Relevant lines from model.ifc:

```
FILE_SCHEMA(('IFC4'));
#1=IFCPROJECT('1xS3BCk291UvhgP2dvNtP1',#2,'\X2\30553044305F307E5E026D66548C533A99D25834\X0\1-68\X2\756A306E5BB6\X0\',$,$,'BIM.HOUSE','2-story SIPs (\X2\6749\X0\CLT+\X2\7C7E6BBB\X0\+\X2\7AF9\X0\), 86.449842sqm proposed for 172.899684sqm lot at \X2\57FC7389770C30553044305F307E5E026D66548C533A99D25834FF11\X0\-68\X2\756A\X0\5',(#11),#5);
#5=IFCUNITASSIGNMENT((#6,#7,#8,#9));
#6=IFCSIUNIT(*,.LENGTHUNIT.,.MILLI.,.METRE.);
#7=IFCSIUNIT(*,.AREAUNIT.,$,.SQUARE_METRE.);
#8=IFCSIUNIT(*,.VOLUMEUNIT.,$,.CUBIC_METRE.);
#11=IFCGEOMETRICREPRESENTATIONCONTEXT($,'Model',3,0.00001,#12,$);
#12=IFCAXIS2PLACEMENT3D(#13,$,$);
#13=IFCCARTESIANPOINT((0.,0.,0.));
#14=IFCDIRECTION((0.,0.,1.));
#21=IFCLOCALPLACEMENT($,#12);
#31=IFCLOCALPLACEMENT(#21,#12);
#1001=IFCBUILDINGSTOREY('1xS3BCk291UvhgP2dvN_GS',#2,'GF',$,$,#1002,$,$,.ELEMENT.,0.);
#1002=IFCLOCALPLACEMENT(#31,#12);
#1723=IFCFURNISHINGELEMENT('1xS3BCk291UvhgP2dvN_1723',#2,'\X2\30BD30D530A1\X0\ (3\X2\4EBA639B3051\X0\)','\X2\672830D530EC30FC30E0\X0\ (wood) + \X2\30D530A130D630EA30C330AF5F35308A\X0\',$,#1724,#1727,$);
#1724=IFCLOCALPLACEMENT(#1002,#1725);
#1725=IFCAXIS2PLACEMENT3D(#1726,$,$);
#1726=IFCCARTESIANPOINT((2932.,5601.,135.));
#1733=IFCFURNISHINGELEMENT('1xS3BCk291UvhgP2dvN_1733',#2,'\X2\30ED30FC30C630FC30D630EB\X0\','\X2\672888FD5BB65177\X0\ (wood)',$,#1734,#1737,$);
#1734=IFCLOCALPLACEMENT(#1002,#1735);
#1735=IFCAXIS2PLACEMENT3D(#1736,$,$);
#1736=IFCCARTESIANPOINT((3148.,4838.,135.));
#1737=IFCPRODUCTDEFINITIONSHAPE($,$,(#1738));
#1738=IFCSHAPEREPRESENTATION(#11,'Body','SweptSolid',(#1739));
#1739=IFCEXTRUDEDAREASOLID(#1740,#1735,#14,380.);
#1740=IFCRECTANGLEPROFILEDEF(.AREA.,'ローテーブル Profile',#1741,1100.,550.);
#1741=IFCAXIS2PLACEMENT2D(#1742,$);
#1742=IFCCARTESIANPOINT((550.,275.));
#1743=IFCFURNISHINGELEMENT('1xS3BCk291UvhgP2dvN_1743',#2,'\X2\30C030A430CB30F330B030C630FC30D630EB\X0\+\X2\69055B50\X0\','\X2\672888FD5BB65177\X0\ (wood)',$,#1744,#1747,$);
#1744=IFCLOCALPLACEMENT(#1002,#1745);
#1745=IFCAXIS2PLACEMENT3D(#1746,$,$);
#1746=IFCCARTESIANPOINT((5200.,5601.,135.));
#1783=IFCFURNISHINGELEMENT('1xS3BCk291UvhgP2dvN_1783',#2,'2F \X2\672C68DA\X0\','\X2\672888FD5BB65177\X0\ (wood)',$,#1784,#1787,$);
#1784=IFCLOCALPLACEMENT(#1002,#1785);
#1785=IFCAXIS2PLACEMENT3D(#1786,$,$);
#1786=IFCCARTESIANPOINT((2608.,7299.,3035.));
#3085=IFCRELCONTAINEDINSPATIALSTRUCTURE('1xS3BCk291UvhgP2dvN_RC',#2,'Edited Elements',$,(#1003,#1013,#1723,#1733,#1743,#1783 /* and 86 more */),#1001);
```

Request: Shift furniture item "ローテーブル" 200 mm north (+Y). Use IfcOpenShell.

```python
import ifcopenshell
import ifcopenshell.api.geometry
import ifcopenshell.util.placement
import ifcopenshell.util.unit

model = ifcopenshell.open("model.ifc")
unit_scale = ifcopenshell.util.unit.calculate_unit_scale(model)

item = model.by_id(1733)
matrix = ifcopenshell.util.placement.get_local_placement(item.ObjectPlacement)
matrix[1, 3] += 0.2 / unit_scale
ifcopenshell.api.geometry.edit_object_placement(model, product=item, matrix=matrix, is_si=False)

print(ifcopenshell.util.placement.get_local_placement(item.ObjectPlacement).round(3) + 0.0)

model.write("model_rev.ifc")
```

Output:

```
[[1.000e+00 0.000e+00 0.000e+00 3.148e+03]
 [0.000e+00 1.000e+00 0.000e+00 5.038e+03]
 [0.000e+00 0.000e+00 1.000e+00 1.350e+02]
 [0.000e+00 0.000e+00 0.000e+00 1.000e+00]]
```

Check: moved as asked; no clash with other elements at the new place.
